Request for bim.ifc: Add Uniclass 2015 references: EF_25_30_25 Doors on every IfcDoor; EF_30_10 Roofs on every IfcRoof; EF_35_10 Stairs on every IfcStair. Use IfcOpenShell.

First a look at what the model holds.

```python
import ifcopenshell

model = ifcopenshell.open("bim.ifc")
print(model.schema)
print("classifications:", [c.Name for c in model.by_type("IfcClassification")])
for ifc_class in ("IfcDoor", "IfcRoof", "IfcStair", "IfcWall", "IfcWindow"):
    print(ifc_class, len(model.by_type(ifc_class)))
```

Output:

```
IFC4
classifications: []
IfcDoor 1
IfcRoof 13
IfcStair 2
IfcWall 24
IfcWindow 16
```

```python
import ifcopenshell
import ifcopenshell.api.classification

model = ifcopenshell.open("bim.ifc")

system = ifcopenshell.api.classification.add_classification(model, classification="Uniclass 2015")

codes = {
    "IfcDoor": ("EF_25_30_25", "Doors"),
    "IfcRoof": ("EF_30_10", "Roofs"),
    "IfcStair": ("EF_35_10", "Stairs"),
}
for ifc_class, (code, name) in codes.items():
    products = model.by_type(ifc_class)
    ifcopenshell.api.classification.add_reference(
        model, products=products, classification=system, identification=code, name=name
    )
    print(code, len(products))

model.write("bim_v2.ifc")
```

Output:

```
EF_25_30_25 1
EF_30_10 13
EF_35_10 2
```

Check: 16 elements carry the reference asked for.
